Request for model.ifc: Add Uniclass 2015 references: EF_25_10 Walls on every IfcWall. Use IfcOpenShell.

First a look at what the model holds.

```python
import ifcopenshell

model = ifcopenshell.open("model.ifc")
print(model.schema)
print("classifications:", [c.Name for c in model.by_type("IfcClassification")])
for ifc_class in ("IfcDoor", "IfcRoof", "IfcStair", "IfcWall", "IfcWindow"):
    print(ifc_class, len(model.by_type(ifc_class)))
```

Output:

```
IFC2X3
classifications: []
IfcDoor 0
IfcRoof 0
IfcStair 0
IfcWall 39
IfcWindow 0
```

```python
import ifcopenshell
import ifcopenshell.api.classification

model = ifcopenshell.open("model.ifc")

# IFC2X3 requires Source and Edition and has no link from the project to the system.
system = model.create_entity("IfcClassification", Source="NBS", Edition="2015", Name="Uniclass 2015")

codes = {
    "IfcWall": ("EF_25_10", "Walls"),
}
for ifc_class, (code, name) in codes.items():
    products = model.by_type(ifc_class)
    ifcopenshell.api.classification.add_reference(
        model, products=products, classification=system, identification=code, name=name
    )
    print(code, len(products))

model.write("model-out.ifc")
```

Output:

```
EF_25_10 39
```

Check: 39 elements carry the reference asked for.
